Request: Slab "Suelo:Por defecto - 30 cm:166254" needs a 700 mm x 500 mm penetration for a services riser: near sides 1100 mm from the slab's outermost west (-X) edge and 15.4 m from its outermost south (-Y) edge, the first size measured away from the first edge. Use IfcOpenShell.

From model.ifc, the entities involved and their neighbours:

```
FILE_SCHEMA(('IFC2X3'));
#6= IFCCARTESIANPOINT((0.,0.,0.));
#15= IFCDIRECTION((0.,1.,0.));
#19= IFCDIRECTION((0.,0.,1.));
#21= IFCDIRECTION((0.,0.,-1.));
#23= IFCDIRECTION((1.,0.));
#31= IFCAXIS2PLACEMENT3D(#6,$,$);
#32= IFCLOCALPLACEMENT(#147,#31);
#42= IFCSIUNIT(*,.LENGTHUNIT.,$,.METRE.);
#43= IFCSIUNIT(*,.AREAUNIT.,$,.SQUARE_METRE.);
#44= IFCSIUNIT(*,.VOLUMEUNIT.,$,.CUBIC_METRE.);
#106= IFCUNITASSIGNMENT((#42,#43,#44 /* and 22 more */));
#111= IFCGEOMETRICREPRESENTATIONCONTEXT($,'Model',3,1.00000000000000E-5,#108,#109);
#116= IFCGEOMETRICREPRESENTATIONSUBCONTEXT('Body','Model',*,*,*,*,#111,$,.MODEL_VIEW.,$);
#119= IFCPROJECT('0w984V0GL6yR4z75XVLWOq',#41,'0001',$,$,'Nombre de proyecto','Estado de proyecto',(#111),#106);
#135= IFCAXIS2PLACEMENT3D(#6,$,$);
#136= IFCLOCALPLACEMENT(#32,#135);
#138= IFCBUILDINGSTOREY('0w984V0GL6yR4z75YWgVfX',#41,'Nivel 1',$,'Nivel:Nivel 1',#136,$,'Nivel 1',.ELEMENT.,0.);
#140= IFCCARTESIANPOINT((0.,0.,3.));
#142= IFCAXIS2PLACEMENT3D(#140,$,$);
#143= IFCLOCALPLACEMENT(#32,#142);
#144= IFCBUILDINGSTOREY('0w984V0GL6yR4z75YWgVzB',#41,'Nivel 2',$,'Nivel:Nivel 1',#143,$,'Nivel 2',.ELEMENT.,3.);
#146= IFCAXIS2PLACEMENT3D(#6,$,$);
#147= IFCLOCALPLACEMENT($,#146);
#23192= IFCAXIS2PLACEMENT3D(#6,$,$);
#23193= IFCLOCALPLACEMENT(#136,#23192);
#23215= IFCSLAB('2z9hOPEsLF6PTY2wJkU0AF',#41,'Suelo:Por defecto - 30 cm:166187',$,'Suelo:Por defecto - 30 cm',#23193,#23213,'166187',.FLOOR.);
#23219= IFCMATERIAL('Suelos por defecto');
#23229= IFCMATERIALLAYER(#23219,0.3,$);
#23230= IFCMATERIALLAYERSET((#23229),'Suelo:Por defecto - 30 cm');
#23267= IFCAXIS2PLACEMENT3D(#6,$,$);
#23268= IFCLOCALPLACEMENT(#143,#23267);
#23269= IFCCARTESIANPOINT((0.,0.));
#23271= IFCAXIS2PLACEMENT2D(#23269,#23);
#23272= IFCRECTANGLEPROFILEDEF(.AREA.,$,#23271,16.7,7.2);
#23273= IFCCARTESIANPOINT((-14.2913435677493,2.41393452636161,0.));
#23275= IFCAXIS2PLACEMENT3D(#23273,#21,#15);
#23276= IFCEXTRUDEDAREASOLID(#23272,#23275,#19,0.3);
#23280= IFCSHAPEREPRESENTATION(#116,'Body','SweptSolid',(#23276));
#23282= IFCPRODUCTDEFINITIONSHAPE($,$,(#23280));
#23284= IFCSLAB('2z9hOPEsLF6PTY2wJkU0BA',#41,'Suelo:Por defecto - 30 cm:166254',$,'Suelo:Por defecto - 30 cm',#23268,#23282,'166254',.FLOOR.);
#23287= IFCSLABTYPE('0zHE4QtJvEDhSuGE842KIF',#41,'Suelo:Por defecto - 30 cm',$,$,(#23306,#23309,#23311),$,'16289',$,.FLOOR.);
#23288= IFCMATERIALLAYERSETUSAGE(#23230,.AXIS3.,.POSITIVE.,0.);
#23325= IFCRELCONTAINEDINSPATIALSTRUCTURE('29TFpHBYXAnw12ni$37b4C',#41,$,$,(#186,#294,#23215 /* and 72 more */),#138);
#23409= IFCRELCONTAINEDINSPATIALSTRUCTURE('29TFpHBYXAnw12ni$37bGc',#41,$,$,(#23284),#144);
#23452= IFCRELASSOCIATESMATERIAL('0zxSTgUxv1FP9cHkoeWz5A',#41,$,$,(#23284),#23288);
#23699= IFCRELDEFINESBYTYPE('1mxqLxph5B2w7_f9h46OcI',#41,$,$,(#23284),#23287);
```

```python
import numpy as np
import ifcopenshell
import ifcopenshell.api.feature
import ifcopenshell.api.geometry
import ifcopenshell.api.root
import ifcopenshell.geom
import ifcopenshell.util.placement
import ifcopenshell.util.representation
import ifcopenshell.util.shape
import ifcopenshell.util.unit

model = ifcopenshell.open("model.ifc")
unit_scale = ifcopenshell.util.unit.calculate_unit_scale(model)
settings = ifcopenshell.geom.settings()


def volume(element):
    """Net volume in cubic metres, openings subtracted."""
    shape = ifcopenshell.geom.create_shape(settings, element)
    return ifcopenshell.util.shape.get_volume(shape.geometry)


slab = model.by_guid("2z9hOPEsLF6PTY2wJkU0BA")
before = volume(slab)

# Extent in the slab's own axes, in metres. The edges named are its -X and -Y sides.
slab_shape = ifcopenshell.geom.create_shape(settings, slab)
vertices = ifcopenshell.util.shape.get_vertices(slab_shape.geometry)
x_min, y_min, bottom = vertices.min(axis=0)
top = vertices[:, 2].max()

opening = ifcopenshell.api.root.create_entity(model, ifc_class="IfcOpeningElement", name="Services riser opening")
context = ifcopenshell.util.representation.get_context(model, "Model", "Body", "MODEL_VIEW")
width, depth = 0.7, 0.5
outline = [(0.0, 0.0), (width, 0.0), (width, depth), (0.0, depth), (0.0, 0.0)]
# Overshoot both faces by 50 mm so the cut is clean.
shape = ifcopenshell.api.geometry.add_slab_representation(
    model, context=context, depth=top - bottom + 0.1, polyline=outline
)
ifcopenshell.api.geometry.assign_representation(model, product=opening, representation=shape)

matrix = ifcopenshell.util.placement.get_local_placement(slab.ObjectPlacement)
matrix[:, 3] = matrix @ np.append(np.array([x_min + 1.1, y_min + 15.4, bottom - 0.05]) / unit_scale, 1.0)
ifcopenshell.api.geometry.edit_object_placement(model, product=opening, matrix=matrix, is_si=False)
ifcopenshell.api.feature.add_feature(model, feature=opening, element=slab)

after = volume(slab)

print(f"slab volume {before:.3f} -> {after:.3f} m3")

model.write("model_edited.ifc")
```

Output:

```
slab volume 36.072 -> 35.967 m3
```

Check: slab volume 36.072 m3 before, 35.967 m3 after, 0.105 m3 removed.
